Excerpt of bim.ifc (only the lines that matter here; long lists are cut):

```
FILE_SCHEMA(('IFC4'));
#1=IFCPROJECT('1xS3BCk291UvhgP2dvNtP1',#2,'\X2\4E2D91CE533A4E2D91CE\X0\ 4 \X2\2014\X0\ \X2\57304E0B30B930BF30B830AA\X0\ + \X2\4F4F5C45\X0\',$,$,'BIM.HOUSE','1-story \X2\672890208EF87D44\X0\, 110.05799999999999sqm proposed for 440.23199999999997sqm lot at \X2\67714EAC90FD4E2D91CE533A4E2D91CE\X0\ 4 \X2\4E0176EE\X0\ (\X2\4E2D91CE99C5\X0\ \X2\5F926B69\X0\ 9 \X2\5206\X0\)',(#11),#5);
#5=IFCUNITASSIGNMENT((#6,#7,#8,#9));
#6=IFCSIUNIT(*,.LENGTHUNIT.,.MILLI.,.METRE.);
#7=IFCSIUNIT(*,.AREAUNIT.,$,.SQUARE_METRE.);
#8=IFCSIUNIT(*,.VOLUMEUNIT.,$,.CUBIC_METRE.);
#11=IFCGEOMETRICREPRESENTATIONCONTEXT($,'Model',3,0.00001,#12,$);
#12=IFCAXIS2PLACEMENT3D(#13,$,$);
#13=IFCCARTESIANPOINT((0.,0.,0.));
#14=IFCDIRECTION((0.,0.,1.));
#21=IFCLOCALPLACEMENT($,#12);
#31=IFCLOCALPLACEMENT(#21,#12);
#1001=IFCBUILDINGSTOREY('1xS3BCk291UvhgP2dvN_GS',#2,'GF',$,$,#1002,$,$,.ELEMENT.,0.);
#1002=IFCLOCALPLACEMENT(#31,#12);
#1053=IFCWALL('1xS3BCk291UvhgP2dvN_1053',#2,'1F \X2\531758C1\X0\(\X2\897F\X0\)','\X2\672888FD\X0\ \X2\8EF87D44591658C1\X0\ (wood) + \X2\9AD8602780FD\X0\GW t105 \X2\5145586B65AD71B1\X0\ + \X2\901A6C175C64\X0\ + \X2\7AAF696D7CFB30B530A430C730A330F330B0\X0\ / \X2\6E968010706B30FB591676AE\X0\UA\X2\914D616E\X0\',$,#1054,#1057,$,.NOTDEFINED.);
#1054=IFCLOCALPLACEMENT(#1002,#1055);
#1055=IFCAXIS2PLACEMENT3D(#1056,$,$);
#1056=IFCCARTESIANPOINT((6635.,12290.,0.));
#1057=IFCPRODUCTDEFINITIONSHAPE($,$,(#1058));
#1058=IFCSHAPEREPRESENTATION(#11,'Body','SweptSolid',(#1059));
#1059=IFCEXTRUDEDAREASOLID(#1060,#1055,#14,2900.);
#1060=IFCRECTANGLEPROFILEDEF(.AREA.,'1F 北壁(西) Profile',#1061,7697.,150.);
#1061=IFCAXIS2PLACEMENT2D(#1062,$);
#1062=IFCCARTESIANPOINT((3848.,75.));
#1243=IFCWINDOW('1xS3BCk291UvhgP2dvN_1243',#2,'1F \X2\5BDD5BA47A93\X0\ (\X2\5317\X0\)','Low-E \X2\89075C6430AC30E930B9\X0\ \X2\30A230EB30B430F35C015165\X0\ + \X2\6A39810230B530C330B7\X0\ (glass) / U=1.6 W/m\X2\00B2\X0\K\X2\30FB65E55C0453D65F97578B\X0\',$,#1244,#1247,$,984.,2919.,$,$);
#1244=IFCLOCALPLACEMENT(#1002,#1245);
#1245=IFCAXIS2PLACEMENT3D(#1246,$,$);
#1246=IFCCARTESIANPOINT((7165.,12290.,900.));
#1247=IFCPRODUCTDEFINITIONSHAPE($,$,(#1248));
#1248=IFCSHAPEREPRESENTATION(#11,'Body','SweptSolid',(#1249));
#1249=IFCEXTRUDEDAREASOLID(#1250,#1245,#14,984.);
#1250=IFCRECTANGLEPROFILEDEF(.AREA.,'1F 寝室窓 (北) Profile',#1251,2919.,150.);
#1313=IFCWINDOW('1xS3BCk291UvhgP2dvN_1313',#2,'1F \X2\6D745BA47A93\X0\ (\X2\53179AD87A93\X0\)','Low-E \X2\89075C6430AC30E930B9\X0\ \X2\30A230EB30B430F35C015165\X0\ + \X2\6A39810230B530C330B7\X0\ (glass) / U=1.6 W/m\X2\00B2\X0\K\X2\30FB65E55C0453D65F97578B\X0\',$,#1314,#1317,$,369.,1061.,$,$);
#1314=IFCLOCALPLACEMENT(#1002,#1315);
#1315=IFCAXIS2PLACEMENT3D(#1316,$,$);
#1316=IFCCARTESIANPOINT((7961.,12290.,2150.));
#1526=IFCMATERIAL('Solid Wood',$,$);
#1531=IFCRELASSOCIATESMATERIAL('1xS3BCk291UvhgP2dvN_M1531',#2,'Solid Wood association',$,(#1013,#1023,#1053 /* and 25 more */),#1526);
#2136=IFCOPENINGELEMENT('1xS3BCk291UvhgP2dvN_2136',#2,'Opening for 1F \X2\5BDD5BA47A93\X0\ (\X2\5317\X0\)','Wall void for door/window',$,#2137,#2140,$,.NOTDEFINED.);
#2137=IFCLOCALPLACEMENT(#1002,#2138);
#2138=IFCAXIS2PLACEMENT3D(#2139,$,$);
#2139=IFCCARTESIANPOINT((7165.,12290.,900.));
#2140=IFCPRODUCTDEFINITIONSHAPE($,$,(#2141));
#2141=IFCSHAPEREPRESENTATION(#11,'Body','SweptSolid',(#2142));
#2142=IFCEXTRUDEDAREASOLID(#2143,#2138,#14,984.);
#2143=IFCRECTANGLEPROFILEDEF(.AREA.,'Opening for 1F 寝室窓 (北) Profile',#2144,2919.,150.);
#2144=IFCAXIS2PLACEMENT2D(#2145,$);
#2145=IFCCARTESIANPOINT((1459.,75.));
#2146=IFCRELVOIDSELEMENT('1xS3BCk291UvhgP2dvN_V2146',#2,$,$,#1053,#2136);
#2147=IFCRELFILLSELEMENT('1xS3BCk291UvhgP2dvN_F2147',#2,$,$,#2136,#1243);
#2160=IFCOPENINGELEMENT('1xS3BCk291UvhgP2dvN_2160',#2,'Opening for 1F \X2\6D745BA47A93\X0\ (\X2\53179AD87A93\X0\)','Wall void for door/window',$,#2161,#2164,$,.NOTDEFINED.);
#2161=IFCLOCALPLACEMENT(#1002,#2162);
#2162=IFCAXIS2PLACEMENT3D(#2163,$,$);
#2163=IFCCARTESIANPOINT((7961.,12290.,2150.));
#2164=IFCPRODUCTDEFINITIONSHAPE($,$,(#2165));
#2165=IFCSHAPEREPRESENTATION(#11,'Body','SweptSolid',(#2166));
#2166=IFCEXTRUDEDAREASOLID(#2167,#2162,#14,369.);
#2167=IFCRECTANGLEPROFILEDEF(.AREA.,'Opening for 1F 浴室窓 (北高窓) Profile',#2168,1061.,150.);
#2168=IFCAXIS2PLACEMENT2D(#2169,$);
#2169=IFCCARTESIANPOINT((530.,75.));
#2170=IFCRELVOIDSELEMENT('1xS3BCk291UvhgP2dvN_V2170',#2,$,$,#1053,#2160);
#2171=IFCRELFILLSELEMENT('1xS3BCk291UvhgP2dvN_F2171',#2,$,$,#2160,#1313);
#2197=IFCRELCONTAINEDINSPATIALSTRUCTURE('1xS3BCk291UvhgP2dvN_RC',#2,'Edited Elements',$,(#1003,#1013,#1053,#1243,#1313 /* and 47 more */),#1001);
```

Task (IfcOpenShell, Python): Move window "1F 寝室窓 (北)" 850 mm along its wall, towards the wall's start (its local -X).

```python
import ifcopenshell
import ifcopenshell.api.geometry
import ifcopenshell.util.placement

model = ifcopenshell.open("bim.ifc")

window = model.by_id(1243)
opening = window.FillsVoids[0].RelatingOpeningElement
wall = opening.VoidsElements[0].RelatingBuildingElement

wall_matrix = ifcopenshell.util.placement.get_local_placement(wall.ObjectPlacement)
shift = wall_matrix[:3, 0] * -850.0
before = ifcopenshell.util.placement.get_local_placement(window.ObjectPlacement)[:3, 3].copy()

# The window is not placed relative to its opening, so move both.
for product in (opening, window):
    matrix = ifcopenshell.util.placement.get_local_placement(product.ObjectPlacement)
    matrix[:3, 3] += shift
    ifcopenshell.api.geometry.edit_object_placement(model, product=product, matrix=matrix, is_si=False)

after = ifcopenshell.util.placement.get_local_placement(window.ObjectPlacement)[:3, 3]
print("window moved by", (after - before).round(3) + 0.0)

model.write("bim_rev.ifc")
```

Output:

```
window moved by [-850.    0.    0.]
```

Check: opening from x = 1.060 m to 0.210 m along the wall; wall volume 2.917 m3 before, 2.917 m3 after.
